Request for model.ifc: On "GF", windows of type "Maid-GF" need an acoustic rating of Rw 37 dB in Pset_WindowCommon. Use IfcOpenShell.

First a look at what the model holds.

```python
import ifcopenshell
import ifcopenshell.util.element

model = ifcopenshell.open("model.ifc")
print(model.schema)
storey = next(s for s in model.by_type("IfcBuildingStorey") if s.Name == "GF")
windows = [e for e in ifcopenshell.util.element.get_decomposition(storey) if e.is_a("IfcWindow")]
seen = {}
for e in windows:
    element_type = ifcopenshell.util.element.get_type(e)
    key = (element_type.Name if element_type != e and element_type else None, ifcopenshell.util.element.get_pset(e, "Pset_WindowCommon", "AcousticRating"))
    seen[key] = seen.get(key, 0) + 1
for (name, value), count in sorted(seen.items(), key=str):
    print(count, "x", name, "|", value)
```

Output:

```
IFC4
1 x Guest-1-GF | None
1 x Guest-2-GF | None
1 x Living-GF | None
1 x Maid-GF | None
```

```python
import ifcopenshell
import ifcopenshell.api.pset
import ifcopenshell.util.element

model = ifcopenshell.open("model.ifc")

storey = next(s for s in model.by_type("IfcBuildingStorey") if s.Name == "GF")
windows = [e for e in ifcopenshell.util.element.get_decomposition(storey) if e.is_a("IfcWindow")]

count = 0
for e in windows:
    element_type = ifcopenshell.util.element.get_type(e)
    if element_type in (None, e) or element_type.Name != "Maid-GF":
        continue
    # add_pset returns the element's existing set when there is one.
    pset = ifcopenshell.api.pset.add_pset(model, product=e, name="Pset_WindowCommon")
    ifcopenshell.api.pset.edit_pset(model, pset=pset, properties={"AcousticRating": "Rw 37 dB"})
    count += 1

print(count, "windows updated")

model.write("model_edited.ifc")
```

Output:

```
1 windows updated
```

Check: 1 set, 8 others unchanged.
